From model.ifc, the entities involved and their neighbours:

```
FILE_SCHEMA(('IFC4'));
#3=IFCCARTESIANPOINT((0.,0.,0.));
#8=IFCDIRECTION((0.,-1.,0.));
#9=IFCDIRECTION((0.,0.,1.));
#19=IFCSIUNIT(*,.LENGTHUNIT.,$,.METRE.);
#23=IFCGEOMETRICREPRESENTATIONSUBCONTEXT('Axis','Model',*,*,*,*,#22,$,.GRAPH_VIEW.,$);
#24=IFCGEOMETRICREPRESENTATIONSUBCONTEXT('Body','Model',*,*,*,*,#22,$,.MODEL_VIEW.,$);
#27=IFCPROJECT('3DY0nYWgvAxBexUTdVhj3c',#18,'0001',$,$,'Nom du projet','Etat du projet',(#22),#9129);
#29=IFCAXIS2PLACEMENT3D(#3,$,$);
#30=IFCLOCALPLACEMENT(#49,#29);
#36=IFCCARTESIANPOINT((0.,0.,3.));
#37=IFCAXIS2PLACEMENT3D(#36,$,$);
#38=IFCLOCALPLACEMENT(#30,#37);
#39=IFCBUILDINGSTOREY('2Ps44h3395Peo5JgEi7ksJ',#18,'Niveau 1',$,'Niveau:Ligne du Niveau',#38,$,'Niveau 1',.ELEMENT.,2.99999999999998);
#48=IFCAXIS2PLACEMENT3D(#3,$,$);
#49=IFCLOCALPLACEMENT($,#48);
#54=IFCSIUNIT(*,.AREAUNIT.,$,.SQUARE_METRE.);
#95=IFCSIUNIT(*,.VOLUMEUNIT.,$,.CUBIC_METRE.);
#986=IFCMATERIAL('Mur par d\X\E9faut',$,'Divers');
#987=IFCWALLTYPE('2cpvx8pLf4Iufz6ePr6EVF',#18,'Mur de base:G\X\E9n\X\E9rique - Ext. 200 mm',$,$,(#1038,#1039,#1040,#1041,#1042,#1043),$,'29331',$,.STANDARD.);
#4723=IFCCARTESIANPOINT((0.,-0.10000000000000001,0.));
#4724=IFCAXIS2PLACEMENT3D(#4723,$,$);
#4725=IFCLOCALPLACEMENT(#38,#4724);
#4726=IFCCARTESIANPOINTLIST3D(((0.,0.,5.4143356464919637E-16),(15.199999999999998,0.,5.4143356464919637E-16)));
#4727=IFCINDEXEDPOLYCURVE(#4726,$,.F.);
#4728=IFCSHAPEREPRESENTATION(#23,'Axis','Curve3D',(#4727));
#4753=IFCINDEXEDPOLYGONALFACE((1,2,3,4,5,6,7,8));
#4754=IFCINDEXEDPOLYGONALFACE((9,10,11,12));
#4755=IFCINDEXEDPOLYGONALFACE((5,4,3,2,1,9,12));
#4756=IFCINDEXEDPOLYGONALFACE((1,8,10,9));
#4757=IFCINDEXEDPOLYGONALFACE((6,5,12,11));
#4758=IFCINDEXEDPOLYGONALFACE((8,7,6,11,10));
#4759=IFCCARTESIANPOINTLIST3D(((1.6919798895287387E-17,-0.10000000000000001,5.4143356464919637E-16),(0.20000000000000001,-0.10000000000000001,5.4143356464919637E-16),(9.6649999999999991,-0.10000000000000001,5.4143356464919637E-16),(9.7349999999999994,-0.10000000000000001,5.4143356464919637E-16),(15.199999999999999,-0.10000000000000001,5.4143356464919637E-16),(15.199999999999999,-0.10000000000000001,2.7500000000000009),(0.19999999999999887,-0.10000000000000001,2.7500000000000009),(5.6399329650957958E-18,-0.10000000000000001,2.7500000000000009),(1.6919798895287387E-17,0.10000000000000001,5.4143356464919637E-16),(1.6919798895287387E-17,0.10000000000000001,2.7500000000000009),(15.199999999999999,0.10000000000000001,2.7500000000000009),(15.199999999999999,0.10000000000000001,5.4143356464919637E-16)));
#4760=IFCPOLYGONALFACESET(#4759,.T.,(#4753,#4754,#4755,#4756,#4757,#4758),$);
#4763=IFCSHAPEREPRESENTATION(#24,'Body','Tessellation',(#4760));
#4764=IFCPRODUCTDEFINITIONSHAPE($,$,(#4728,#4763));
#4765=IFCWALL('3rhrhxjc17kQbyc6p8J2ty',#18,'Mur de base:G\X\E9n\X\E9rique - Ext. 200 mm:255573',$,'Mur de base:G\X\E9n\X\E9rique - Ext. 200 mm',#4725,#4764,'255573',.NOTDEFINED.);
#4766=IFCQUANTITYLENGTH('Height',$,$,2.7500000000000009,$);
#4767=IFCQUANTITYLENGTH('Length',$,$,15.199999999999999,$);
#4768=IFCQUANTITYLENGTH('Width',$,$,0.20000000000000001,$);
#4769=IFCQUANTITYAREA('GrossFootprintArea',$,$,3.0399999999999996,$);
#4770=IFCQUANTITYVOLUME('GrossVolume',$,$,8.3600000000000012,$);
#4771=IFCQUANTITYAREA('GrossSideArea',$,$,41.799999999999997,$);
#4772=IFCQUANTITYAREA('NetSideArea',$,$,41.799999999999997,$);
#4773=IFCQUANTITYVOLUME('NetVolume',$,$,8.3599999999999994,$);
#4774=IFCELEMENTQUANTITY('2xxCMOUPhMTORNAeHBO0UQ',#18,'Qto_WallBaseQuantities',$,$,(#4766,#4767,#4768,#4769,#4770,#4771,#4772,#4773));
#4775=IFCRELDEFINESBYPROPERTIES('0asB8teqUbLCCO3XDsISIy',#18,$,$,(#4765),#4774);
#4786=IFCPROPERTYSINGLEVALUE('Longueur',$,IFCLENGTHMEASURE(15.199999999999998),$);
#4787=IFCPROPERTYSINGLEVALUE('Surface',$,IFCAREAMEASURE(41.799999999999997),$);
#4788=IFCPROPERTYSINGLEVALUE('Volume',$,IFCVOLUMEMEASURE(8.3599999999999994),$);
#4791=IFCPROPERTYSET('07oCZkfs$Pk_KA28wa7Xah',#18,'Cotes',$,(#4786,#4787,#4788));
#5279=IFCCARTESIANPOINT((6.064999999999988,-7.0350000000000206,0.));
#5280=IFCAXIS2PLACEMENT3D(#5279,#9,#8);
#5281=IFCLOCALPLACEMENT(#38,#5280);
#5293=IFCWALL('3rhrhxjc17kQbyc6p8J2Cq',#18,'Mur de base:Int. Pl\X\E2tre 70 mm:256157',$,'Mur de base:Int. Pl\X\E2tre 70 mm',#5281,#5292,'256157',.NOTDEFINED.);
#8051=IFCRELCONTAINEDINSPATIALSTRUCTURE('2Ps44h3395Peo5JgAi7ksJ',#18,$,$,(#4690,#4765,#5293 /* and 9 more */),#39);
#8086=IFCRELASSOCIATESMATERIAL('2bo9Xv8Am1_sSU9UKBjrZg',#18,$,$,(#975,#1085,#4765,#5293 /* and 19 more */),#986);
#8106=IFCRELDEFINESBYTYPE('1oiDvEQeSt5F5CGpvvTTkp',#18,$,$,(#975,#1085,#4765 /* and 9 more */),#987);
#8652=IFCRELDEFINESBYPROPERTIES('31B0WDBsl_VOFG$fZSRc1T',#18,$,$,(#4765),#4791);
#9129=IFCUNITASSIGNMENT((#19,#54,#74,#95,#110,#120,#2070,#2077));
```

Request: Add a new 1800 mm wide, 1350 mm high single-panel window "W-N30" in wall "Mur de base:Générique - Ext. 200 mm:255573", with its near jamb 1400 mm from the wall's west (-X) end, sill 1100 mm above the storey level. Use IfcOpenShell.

```python
import numpy as np
import ifcopenshell
import ifcopenshell.api.feature
import ifcopenshell.api.geometry
import ifcopenshell.api.pset
import ifcopenshell.api.root
import ifcopenshell.api.spatial
import ifcopenshell.geom
import ifcopenshell.util.element
import ifcopenshell.util.placement
import ifcopenshell.util.representation
import ifcopenshell.util.shape
import ifcopenshell.util.unit

model = ifcopenshell.open("model.ifc")
unit_scale = ifcopenshell.util.unit.calculate_unit_scale(model)
area_scale = ifcopenshell.util.unit.calculate_unit_scale(model, "AREAUNIT")
volume_scale = ifcopenshell.util.unit.calculate_unit_scale(model, "VOLUMEUNIT")
settings = ifcopenshell.geom.settings()


def volume(element):
    """Net volume in cubic metres, openings subtracted."""
    shape = ifcopenshell.geom.create_shape(settings, element)
    return ifcopenshell.util.shape.get_volume(shape.geometry)


wall = model.by_id(4765)
storey = ifcopenshell.util.element.get_container(wall, ifc_class="IfcBuildingStorey")
context = ifcopenshell.util.representation.get_context(model, "Model", "Body", "MODEL_VIEW")
before = volume(wall)

width, height, from_end, sill = 1.8, 1.35, 1.4, 1.1  # metres

# The wall runs along its own X axis, and the end named is its -X end.
wall_shape = ifcopenshell.geom.create_shape(settings, wall)
x, y, z = ifcopenshell.util.shape.get_vertices(wall_shape.geometry).T
start = x.min() + from_end
face, thickness = float(y.min()), float(y.max() - y.min())
wall_matrix = ifcopenshell.util.placement.get_local_placement(wall.ObjectPlacement)
level = ifcopenshell.util.placement.get_local_placement(storey.ObjectPlacement)[2, 3]


def in_wall(x, y):
    """Placement at x, y metres in the wall's axes, at sill height."""
    matrix = wall_matrix.copy()
    matrix[:, 3] = wall_matrix @ np.array([x / unit_scale, y / unit_scale, 0.0, 1.0])
    matrix[2, 3] = level + sill / unit_scale
    return matrix


# Opening: a box that overshoots both wall faces by 50 mm.
opening = ifcopenshell.api.root.create_entity(model, ifc_class="IfcOpeningElement", predefined_type="OPENING")
box = ifcopenshell.api.geometry.add_wall_representation(
    model, context=context, length=width, height=height, thickness=thickness + 0.1
)
ifcopenshell.api.geometry.assign_representation(model, product=opening, representation=box)
ifcopenshell.api.geometry.edit_object_placement(model, product=opening, matrix=in_wall(start, face - 0.05), is_si=False)
ifcopenshell.api.feature.add_feature(model, feature=opening, element=wall)

window = ifcopenshell.api.root.create_entity(model, ifc_class="IfcWindow", name="W-N30", predefined_type="WINDOW")
window.OverallWidth, window.OverallHeight = width / unit_scale, height / unit_scale
window.PartitioningType = "SINGLE_PANEL"
body = ifcopenshell.api.geometry.add_window_representation(
    model,
    context=context,
    overall_width=window.OverallWidth,
    overall_height=window.OverallHeight,
    partition_type="SINGLE_PANEL",
)
ifcopenshell.api.geometry.assign_representation(model, product=window, representation=body)
ifcopenshell.api.spatial.assign_container(model, products=[window], relating_structure=storey)
ifcopenshell.api.feature.add_filling(model, opening=opening, element=window)

# Centre the window in the wall's thickness.
ifcopenshell.api.geometry.edit_object_placement(model, product=window, matrix=in_wall(start, face), is_si=False)
window_shape = ifcopenshell.geom.create_shape(settings, window)
depth = ifcopenshell.util.shape.get_vertices(window_shape.geometry)[:, 1]
offset = face + thickness / 2 - (depth.min() + depth.max()) / 2
ifcopenshell.api.geometry.edit_object_placement(model, product=window, matrix=in_wall(start, offset), is_si=False)

after = volume(wall)

# Update the wall's stored quantities.
qto = model.by_id(ifcopenshell.util.element.get_pset(wall, "Qto_WallBaseQuantities", should_inherit=False)["id"])
ifcopenshell.api.pset.edit_qto(model, qto=qto, properties={
    "NetSideArea": after / thickness / area_scale,
    "NetVolume": after / volume_scale,
})
pset = model.by_id(ifcopenshell.util.element.get_pset(wall, "Cotes", should_inherit=False)["id"])
ifcopenshell.api.pset.edit_pset(model, pset=pset, properties={
    "Surface": model.create_entity("IfcAreaMeasure", after / thickness / area_scale),
    "Volume": model.create_entity("IfcVolumeMeasure", after / volume_scale),
})

print(f"wall volume {before:.3f} -> {after:.3f} m3")

model.write("model_v2.ifc")
```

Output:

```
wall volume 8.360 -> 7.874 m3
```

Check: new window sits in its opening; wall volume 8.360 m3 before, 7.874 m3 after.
